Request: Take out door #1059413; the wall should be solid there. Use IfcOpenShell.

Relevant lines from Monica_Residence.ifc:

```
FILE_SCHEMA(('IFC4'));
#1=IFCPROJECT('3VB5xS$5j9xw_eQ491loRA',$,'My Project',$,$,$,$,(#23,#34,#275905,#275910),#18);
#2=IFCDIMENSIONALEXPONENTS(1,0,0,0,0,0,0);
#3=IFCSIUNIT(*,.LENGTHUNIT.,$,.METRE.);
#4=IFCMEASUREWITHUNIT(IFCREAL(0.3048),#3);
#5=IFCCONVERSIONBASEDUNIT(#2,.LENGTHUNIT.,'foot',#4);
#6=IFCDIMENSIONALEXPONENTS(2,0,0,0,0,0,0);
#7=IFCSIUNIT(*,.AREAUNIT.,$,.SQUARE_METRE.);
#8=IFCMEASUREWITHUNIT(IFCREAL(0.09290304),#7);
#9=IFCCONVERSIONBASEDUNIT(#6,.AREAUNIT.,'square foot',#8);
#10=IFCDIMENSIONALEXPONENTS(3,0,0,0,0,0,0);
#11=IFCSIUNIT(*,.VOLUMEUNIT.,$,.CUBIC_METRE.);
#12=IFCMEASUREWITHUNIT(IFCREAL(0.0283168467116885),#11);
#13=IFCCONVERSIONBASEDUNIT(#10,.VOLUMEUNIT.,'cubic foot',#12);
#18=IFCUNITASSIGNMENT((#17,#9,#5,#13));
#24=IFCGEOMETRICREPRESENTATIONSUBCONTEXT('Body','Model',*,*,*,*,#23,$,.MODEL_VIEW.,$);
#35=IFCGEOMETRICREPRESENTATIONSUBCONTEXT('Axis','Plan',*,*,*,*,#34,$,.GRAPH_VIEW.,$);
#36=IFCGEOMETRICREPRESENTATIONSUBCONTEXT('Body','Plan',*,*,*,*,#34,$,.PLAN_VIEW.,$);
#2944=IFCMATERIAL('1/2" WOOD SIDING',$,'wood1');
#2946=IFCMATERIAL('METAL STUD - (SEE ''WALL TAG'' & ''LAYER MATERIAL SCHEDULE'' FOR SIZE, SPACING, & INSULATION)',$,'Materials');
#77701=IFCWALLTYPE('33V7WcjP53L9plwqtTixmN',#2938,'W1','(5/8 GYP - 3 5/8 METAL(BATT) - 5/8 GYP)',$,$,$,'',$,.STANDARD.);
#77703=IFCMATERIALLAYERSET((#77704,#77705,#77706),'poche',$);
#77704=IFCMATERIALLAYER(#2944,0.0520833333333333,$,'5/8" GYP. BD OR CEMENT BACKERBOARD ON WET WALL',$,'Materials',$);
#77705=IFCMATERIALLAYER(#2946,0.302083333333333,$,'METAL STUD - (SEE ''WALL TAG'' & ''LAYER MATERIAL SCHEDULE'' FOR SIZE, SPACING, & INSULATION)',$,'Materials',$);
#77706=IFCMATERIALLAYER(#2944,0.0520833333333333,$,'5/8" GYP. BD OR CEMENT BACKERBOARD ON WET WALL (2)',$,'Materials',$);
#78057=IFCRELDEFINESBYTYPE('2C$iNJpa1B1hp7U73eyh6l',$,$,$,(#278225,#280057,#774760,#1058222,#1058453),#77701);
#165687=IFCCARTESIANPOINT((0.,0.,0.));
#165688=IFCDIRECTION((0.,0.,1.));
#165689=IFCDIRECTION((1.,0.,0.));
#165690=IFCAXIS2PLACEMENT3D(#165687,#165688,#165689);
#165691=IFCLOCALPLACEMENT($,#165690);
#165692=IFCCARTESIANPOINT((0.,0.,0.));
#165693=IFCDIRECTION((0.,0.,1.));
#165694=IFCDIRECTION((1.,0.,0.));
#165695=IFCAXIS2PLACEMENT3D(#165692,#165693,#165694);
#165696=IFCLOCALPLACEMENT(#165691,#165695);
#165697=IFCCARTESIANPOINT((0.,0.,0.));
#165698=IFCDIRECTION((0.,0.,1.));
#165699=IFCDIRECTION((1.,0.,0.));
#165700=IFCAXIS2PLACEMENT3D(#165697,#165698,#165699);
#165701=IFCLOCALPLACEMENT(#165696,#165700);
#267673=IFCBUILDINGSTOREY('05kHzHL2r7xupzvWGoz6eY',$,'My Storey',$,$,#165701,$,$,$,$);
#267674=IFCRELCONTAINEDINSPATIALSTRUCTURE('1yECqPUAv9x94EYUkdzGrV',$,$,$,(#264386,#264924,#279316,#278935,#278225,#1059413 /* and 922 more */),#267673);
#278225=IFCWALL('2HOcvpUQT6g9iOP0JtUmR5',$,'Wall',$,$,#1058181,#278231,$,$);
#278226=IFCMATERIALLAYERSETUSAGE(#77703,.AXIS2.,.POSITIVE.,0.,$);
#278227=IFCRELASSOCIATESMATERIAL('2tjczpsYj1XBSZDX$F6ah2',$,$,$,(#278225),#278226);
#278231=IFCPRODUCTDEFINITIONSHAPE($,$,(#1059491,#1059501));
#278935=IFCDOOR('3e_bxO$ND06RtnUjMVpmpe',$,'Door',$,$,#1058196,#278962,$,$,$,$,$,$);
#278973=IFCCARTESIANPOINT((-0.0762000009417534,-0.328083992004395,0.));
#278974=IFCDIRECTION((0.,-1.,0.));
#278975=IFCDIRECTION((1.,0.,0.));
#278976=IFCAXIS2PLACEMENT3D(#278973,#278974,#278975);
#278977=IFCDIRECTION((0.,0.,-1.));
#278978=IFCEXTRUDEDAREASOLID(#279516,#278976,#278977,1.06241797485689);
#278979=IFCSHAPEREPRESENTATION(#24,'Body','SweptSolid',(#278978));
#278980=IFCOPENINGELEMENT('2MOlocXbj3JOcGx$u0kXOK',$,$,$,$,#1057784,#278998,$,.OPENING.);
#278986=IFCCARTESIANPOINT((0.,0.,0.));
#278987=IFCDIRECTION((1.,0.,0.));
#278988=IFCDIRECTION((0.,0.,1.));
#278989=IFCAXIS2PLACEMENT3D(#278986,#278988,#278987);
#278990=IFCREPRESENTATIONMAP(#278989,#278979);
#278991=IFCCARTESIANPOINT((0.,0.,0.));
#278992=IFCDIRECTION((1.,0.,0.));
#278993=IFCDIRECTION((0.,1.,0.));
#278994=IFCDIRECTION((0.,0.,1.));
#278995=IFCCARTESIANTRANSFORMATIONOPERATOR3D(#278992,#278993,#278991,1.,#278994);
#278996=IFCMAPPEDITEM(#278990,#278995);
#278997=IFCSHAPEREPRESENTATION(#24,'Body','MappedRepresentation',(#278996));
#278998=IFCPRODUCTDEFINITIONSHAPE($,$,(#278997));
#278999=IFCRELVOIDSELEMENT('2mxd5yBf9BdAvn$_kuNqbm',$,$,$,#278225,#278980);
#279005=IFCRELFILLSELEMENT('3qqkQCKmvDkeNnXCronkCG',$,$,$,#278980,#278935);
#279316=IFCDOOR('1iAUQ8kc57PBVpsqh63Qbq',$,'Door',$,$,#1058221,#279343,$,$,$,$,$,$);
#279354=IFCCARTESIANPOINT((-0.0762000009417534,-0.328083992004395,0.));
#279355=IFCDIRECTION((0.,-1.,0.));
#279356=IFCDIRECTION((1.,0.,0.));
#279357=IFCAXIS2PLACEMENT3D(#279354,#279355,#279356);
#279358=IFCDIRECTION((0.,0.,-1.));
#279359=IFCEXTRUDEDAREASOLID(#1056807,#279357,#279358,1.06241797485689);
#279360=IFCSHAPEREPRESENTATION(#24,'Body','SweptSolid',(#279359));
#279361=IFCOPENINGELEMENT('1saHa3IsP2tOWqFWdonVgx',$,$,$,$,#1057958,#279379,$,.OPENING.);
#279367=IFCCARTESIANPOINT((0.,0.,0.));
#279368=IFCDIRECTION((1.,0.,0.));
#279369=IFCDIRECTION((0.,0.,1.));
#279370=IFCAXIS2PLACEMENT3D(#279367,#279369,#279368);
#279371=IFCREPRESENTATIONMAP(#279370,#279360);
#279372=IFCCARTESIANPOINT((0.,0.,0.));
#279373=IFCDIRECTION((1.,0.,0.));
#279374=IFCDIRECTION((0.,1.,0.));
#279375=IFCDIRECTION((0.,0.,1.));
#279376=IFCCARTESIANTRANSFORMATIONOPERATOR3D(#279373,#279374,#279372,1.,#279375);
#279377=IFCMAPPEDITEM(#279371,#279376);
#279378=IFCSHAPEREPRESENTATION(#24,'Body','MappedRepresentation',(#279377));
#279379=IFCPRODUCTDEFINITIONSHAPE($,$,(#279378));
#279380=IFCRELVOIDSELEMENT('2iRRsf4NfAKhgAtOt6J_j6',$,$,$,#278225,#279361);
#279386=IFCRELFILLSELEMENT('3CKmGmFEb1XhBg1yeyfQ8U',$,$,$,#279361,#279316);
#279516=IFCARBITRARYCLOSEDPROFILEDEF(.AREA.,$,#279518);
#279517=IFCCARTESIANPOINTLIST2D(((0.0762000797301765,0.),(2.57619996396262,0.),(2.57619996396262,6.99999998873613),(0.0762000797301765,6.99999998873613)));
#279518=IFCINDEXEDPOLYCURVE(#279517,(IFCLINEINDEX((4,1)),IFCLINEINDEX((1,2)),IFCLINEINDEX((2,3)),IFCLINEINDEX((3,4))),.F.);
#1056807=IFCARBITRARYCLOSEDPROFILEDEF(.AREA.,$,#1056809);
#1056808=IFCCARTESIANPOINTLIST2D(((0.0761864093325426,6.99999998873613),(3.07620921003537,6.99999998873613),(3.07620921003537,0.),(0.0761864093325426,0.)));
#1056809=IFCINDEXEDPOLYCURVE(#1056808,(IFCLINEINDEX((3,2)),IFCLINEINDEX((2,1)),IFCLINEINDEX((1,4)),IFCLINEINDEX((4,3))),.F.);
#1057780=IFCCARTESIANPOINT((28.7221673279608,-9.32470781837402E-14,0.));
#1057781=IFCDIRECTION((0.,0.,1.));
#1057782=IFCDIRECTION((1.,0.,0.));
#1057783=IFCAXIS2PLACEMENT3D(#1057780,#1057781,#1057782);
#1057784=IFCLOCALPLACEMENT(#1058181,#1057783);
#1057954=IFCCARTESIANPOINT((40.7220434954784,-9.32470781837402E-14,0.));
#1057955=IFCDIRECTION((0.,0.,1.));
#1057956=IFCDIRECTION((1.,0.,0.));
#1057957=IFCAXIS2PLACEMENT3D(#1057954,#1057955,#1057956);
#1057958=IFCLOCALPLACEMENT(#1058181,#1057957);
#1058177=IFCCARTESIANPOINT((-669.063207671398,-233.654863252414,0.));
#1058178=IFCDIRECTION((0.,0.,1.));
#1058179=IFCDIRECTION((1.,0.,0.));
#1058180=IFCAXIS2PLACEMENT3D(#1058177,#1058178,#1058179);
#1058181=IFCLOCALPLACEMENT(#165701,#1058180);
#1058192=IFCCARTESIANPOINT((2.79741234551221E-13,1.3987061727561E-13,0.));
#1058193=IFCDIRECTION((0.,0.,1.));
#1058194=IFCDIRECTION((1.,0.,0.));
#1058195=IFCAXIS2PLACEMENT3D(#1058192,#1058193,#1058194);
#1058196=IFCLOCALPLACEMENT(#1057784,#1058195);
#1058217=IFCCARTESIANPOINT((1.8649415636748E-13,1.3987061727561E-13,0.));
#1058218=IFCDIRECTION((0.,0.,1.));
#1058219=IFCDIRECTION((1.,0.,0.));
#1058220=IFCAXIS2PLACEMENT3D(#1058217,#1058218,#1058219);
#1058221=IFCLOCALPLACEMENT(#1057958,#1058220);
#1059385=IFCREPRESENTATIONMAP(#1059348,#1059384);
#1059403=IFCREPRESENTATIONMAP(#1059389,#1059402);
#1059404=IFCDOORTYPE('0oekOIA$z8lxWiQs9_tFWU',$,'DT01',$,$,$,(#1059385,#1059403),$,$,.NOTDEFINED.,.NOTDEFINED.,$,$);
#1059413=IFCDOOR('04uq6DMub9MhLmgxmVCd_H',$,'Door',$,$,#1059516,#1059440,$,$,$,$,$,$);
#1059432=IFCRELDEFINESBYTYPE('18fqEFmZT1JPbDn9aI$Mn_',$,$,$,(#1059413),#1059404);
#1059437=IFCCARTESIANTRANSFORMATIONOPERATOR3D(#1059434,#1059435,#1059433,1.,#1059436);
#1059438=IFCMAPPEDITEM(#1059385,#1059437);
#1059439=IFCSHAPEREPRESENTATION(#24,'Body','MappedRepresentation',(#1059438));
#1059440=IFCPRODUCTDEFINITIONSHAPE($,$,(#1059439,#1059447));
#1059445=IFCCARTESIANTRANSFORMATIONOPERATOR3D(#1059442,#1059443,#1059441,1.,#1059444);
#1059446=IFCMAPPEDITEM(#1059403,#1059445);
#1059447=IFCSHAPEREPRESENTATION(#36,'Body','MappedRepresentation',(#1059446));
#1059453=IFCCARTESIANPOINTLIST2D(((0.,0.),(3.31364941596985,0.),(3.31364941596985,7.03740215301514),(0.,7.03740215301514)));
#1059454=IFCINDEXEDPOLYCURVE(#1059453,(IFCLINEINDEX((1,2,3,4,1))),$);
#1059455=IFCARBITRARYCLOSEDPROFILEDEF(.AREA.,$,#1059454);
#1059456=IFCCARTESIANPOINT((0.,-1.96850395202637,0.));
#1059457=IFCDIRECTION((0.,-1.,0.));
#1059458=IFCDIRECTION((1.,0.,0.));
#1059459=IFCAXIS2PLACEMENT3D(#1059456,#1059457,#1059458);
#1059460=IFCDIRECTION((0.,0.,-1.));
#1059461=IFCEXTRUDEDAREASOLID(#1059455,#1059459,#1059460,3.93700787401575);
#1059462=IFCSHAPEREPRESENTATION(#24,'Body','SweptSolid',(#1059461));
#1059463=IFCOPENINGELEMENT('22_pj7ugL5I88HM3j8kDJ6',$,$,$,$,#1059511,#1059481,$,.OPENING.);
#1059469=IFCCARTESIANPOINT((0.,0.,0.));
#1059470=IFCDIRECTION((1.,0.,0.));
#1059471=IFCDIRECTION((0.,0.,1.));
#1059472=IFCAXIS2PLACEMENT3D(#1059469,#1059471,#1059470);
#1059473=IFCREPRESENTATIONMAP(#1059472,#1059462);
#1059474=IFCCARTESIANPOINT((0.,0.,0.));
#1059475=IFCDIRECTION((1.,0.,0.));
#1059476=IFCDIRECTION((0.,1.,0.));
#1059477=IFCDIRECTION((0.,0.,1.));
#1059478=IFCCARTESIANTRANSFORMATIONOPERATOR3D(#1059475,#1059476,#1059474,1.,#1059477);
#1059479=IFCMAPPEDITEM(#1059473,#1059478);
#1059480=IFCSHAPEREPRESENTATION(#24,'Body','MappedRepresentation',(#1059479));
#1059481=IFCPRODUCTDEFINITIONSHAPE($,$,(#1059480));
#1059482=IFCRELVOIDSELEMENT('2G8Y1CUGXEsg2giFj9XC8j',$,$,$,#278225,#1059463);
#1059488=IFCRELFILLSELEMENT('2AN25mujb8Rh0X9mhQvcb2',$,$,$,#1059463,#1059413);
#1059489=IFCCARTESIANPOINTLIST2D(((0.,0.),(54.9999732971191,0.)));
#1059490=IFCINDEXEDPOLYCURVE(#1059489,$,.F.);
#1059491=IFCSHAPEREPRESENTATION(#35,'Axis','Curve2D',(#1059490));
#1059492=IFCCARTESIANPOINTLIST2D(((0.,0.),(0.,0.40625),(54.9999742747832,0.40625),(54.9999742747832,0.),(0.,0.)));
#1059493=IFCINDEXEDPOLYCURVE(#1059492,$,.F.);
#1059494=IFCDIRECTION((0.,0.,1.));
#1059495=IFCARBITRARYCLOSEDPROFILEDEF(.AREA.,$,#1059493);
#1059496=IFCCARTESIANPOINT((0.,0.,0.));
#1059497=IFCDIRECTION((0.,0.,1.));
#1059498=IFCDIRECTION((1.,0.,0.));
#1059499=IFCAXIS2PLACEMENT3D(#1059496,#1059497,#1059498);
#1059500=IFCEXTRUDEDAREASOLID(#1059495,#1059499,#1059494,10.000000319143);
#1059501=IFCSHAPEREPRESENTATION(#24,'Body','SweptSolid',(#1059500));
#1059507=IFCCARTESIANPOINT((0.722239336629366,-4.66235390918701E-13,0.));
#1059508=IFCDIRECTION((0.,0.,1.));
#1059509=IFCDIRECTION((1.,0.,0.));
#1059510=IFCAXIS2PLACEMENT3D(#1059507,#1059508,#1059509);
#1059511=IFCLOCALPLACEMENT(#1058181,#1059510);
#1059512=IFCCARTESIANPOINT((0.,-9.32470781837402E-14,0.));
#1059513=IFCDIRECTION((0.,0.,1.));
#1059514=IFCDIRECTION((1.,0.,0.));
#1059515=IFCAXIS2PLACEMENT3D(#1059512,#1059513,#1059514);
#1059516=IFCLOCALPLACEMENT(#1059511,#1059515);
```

```python
import ifcopenshell
import ifcopenshell.api.feature
import ifcopenshell.api.root
import ifcopenshell.geom
import ifcopenshell.util.shape

model = ifcopenshell.open("Monica_Residence.ifc")
settings = ifcopenshell.geom.settings()


def volume(element):
    """Net volume in cubic metres, openings subtracted."""
    shape = ifcopenshell.geom.create_shape(settings, element)
    return ifcopenshell.util.shape.get_volume(shape.geometry)


door = model.by_guid("04uq6DMub9MhLmgxmVCd_H")
opening = door.FillsVoids[0].RelatingOpeningElement
wall = opening.VoidsElements[0].RelatingBuildingElement
before = volume(wall)

ifcopenshell.api.root.remove_product(model, product=door)
ifcopenshell.api.feature.remove_feature(model, feature=opening)

after = volume(wall)

print(f"wall volume {before:.3f} -> {after:.3f} m3")

model.write("Monica_Residence_rev.ifc")
```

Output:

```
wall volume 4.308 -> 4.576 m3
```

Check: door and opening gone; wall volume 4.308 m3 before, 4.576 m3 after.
